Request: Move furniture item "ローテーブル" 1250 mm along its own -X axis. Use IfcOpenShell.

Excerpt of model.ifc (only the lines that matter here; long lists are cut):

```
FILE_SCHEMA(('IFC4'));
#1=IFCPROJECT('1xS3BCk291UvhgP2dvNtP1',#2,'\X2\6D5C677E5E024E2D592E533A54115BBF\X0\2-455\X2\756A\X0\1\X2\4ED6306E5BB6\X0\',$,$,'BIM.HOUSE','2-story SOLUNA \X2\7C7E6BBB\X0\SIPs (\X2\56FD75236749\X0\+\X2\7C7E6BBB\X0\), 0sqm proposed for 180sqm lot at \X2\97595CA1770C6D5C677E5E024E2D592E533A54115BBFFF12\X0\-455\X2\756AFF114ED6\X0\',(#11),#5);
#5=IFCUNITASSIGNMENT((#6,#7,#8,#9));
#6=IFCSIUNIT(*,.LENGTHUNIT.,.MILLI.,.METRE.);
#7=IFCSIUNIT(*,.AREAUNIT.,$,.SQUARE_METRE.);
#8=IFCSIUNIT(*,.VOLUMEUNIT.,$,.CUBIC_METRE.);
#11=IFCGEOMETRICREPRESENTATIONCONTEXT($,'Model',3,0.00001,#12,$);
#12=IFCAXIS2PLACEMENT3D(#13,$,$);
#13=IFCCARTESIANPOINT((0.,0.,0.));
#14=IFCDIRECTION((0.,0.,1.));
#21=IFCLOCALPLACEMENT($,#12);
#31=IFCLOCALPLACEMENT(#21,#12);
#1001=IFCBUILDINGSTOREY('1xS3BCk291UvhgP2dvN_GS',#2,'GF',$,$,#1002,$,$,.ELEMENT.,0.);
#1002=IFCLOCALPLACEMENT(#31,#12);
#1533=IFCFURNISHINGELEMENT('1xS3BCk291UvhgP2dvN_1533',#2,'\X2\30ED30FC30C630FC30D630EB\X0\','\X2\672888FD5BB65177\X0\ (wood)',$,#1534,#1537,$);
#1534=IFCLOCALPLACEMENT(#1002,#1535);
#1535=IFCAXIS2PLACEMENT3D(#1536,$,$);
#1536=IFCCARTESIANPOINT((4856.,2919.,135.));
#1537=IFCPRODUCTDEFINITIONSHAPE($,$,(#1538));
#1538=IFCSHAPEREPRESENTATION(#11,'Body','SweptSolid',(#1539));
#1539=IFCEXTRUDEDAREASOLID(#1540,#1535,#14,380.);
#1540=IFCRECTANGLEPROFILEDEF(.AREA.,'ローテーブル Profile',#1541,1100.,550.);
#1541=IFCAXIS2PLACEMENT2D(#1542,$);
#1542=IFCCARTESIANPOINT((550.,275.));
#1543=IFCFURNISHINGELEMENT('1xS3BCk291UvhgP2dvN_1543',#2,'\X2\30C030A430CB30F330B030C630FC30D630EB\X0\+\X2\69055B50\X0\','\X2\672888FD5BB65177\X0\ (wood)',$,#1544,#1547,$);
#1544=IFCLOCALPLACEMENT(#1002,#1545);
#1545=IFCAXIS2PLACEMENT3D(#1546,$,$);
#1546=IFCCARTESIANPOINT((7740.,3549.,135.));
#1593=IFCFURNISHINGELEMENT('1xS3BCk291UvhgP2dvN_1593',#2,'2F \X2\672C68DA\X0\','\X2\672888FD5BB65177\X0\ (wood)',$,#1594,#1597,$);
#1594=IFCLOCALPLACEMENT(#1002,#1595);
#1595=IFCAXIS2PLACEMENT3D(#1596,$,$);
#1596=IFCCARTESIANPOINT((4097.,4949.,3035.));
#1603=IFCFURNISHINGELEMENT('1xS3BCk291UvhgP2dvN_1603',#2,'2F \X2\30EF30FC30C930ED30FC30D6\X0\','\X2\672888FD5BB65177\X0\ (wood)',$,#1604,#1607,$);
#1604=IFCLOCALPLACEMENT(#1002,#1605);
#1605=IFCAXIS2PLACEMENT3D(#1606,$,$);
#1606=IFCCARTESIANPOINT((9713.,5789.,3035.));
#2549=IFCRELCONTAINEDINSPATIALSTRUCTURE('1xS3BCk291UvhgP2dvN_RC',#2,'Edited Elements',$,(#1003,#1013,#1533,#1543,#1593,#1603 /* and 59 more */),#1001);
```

```python
import ifcopenshell
import ifcopenshell.api.geometry
import ifcopenshell.util.placement

model = ifcopenshell.open("model.ifc")

item = model.by_guid("1xS3BCk291UvhgP2dvN_1533")
matrix = ifcopenshell.util.placement.get_local_placement(item.ObjectPlacement)
matrix[:3, 3] -= matrix[:3, 0] * 1250.0
ifcopenshell.api.geometry.edit_object_placement(model, product=item, matrix=matrix, is_si=False)

print(ifcopenshell.util.placement.get_local_placement(item.ObjectPlacement).round(3) + 0.0)

model.write("model_v2.ifc")
```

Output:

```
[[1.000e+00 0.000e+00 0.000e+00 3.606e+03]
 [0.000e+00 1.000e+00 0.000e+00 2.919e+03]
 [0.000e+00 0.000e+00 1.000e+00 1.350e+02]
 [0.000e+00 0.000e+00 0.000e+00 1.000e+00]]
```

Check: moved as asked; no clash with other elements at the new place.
